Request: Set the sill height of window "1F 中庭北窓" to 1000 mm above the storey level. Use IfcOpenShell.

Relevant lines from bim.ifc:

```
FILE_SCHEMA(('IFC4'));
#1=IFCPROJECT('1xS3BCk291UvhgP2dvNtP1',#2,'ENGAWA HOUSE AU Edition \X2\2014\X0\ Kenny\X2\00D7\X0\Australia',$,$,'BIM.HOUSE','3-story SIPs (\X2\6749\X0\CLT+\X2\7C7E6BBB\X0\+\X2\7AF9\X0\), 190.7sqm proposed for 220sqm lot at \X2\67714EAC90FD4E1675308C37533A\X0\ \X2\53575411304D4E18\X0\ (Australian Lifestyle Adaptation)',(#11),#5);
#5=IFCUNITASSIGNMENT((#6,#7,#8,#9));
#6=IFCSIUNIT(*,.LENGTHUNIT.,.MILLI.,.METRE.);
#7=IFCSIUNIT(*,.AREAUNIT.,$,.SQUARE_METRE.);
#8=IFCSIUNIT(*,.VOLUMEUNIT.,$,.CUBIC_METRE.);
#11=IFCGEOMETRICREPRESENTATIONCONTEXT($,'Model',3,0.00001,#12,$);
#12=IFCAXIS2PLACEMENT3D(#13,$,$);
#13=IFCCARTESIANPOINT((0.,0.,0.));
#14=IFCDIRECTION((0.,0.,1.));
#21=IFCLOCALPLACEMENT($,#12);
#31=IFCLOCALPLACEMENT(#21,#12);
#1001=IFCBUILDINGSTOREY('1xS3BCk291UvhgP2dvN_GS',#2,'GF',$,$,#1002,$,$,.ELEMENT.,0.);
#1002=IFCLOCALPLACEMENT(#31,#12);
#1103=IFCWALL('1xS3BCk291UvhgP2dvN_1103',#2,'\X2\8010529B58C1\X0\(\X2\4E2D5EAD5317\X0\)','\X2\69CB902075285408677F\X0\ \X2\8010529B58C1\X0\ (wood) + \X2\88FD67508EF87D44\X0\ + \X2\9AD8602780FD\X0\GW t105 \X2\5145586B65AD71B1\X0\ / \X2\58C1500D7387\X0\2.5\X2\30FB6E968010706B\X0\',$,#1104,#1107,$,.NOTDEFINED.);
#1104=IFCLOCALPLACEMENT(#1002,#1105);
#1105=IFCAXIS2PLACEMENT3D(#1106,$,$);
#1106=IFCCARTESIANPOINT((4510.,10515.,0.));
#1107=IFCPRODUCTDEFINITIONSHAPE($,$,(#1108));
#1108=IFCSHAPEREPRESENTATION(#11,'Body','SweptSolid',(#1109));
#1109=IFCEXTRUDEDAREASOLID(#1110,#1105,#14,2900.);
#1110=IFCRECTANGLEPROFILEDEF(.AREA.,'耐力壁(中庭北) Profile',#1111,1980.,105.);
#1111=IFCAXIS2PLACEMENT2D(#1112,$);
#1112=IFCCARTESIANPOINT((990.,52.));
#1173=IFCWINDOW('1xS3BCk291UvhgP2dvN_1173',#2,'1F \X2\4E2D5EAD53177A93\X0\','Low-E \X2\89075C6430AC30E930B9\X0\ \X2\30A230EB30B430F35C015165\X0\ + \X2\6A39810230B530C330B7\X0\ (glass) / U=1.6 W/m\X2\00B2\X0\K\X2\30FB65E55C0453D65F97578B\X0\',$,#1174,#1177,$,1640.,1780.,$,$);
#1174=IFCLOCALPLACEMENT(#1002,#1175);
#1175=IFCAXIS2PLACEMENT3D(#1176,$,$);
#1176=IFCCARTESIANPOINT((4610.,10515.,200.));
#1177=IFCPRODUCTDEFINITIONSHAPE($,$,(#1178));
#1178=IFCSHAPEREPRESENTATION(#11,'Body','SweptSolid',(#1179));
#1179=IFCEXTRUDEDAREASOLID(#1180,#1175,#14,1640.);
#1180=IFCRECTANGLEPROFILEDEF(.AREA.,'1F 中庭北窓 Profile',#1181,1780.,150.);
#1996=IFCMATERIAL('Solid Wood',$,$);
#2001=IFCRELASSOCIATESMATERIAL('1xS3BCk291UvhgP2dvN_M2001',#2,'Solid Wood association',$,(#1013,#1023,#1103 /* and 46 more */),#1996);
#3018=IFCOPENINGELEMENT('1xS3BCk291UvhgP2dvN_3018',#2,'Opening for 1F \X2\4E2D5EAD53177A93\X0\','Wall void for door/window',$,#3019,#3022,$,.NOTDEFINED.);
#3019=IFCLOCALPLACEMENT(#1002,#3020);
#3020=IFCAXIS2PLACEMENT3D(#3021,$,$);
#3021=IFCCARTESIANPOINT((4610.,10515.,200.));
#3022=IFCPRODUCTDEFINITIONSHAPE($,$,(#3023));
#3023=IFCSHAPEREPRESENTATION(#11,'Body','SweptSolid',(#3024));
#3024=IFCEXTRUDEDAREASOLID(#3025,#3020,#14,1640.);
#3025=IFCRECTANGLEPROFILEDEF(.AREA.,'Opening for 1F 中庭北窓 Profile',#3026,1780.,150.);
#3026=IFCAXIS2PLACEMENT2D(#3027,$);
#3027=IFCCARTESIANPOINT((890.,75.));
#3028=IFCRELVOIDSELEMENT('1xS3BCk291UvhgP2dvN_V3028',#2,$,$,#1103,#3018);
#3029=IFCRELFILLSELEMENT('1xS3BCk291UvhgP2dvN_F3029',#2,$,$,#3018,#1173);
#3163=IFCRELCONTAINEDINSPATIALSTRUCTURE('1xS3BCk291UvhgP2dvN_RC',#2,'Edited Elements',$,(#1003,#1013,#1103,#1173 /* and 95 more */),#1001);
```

```python
import numpy as np
import ifcopenshell
import ifcopenshell.api.geometry
import ifcopenshell.geom
import ifcopenshell.util.element
import ifcopenshell.util.placement
import ifcopenshell.util.shape
import ifcopenshell.util.unit

model = ifcopenshell.open("bim.ifc")
unit_scale = ifcopenshell.util.unit.calculate_unit_scale(model)

window = model.by_id(1173)
opening = window.FillsVoids[0].RelatingOpeningElement
storey = ifcopenshell.util.element.get_container(window, ifc_class="IfcBuildingStorey")
level = ifcopenshell.util.placement.get_local_placement(storey.ObjectPlacement)[2, 3]

# The opening's origin need not be at the sill, so measure its lowest point.
shape = ifcopenshell.geom.create_shape(ifcopenshell.geom.settings(), opening)
bottom = ifcopenshell.util.shape.get_shape_bottom_elevation(shape, shape.geometry) / unit_scale
dz = level + 1000.0 - bottom

shift = np.array([0.0, 0.0, dz])
# The window is not placed relative to its opening, so move both.
for product in (opening, window):
    matrix = ifcopenshell.util.placement.get_local_placement(product.ObjectPlacement)
    matrix[:3, 3] += shift
    ifcopenshell.api.geometry.edit_object_placement(model, product=product, matrix=matrix, is_si=False)

print(f"moved by {dz * unit_scale:+.3f} m")

model.write("bim_rev.ifc")
```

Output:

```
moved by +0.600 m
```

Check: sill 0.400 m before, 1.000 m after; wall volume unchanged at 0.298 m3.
